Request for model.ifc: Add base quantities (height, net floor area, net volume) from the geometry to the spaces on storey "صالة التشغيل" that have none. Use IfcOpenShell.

First a look at what the model holds.

```python
import ifcopenshell
import ifcopenshell.util.element
import ifcopenshell.util.unit

model = ifcopenshell.open("model.ifc")
print(model.schema)
for unit_type in ("LENGTHUNIT", "AREAUNIT", "VOLUMEUNIT"):
    print(unit_type, ifcopenshell.util.unit.calculate_unit_scale(model, unit_type))
storey = next(s for s in model.by_type("IfcBuildingStorey") if s.Name == "صالة التشغيل")
spaces = [e for e in ifcopenshell.util.element.get_decomposition(storey) if e.is_a("IfcSpace")]
for e in sorted(spaces, key=lambda e: e.id()):
    print(e.id(), e.is_a(), e.Name, list(ifcopenshell.util.element.get_psets(e, qtos_only=True)), sep=" | ")
```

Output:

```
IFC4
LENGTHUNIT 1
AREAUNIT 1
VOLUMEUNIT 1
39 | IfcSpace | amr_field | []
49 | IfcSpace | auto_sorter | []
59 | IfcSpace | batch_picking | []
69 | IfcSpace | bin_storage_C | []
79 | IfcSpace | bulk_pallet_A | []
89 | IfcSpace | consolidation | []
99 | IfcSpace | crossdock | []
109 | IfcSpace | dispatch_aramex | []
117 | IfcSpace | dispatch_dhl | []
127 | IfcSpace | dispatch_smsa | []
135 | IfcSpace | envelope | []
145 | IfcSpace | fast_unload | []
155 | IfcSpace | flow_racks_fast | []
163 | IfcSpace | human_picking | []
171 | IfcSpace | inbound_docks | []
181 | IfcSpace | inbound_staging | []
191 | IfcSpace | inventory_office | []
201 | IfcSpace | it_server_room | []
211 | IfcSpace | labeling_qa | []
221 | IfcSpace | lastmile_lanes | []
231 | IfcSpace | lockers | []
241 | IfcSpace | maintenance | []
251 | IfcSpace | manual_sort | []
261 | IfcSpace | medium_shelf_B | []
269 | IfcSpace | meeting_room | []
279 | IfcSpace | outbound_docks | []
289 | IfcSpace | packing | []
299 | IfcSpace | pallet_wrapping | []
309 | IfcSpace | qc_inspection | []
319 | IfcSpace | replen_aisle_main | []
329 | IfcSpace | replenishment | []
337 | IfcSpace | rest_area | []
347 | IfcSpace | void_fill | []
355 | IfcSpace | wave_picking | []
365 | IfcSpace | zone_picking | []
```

```python
import ifcopenshell
import ifcopenshell.api.pset
import ifcopenshell.geom
import ifcopenshell.util.element
import ifcopenshell.util.shape
import ifcopenshell.util.unit

model = ifcopenshell.open("model.ifc")
unit_scale = ifcopenshell.util.unit.calculate_unit_scale(model)
area_scale = ifcopenshell.util.unit.calculate_unit_scale(model, "AREAUNIT")
volume_scale = ifcopenshell.util.unit.calculate_unit_scale(model, "VOLUMEUNIT")
settings = ifcopenshell.geom.settings()

storey = next(s for s in model.by_type("IfcBuildingStorey") if s.Name == "صالة التشغيل")
spaces = [e for e in ifcopenshell.util.element.get_decomposition(storey) if e.is_a("IfcSpace")]

for e in sorted(spaces, key=lambda e: e.id()):
    if ifcopenshell.util.element.get_psets(e, qtos_only=True, should_inherit=False):
        continue
    # Geometry comes back in metres, in the element's own axes.
    shape = ifcopenshell.geom.create_shape(settings, e)
    values = {
        "Height": ifcopenshell.util.shape.get_z(shape.geometry) / unit_scale,
        "NetFloorArea": ifcopenshell.util.shape.get_footprint_area(shape.geometry) / area_scale,
        "NetVolume": ifcopenshell.util.shape.get_volume(shape.geometry) / volume_scale,
    }
    qto = ifcopenshell.api.pset.add_qto(model, product=e, name="Qto_SpaceBaseQuantities")
    ifcopenshell.api.pset.edit_qto(model, qto=qto, properties=values)
    print(e.id(), {k: round(v, 3) for k, v in values.items()})

model.write("model_rev.ifc")
```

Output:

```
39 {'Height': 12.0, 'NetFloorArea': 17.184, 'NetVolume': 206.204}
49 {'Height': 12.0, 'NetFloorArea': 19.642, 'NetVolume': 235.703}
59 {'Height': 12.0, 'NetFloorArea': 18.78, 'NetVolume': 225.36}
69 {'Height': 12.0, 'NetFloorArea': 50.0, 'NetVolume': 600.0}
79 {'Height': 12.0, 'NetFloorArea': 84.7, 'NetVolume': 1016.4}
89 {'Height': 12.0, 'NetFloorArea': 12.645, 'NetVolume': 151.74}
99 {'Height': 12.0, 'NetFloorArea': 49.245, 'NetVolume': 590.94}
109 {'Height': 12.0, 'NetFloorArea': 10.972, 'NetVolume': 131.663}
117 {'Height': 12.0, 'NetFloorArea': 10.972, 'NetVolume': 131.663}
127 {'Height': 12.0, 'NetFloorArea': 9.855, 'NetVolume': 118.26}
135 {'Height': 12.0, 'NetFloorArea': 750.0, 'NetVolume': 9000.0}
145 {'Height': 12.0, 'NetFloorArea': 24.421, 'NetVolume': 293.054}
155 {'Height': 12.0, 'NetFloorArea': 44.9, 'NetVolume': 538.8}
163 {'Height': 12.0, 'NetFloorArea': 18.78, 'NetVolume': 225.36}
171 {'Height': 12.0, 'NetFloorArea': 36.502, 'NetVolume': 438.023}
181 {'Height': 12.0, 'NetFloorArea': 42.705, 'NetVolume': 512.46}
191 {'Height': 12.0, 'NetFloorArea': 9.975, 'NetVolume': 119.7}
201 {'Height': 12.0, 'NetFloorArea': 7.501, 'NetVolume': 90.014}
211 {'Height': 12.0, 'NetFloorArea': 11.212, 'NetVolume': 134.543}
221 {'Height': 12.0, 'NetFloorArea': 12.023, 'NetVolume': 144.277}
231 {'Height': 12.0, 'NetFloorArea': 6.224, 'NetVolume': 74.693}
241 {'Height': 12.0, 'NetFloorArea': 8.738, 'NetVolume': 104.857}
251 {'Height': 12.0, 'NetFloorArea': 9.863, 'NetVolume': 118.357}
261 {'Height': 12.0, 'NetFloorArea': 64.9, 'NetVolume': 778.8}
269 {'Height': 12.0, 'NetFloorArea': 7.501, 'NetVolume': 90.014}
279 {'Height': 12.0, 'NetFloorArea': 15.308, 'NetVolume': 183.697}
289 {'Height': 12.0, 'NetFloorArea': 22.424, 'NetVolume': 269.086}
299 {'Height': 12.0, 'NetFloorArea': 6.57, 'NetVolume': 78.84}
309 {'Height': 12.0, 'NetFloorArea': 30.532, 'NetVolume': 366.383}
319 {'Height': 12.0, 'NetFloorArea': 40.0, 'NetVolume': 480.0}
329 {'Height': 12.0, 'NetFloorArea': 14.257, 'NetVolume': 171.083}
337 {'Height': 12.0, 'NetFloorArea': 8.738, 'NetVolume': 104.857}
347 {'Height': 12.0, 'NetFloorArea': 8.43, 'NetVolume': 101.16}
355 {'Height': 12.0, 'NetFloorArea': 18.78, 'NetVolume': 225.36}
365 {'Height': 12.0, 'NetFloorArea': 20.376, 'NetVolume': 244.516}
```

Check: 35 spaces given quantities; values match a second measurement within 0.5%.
